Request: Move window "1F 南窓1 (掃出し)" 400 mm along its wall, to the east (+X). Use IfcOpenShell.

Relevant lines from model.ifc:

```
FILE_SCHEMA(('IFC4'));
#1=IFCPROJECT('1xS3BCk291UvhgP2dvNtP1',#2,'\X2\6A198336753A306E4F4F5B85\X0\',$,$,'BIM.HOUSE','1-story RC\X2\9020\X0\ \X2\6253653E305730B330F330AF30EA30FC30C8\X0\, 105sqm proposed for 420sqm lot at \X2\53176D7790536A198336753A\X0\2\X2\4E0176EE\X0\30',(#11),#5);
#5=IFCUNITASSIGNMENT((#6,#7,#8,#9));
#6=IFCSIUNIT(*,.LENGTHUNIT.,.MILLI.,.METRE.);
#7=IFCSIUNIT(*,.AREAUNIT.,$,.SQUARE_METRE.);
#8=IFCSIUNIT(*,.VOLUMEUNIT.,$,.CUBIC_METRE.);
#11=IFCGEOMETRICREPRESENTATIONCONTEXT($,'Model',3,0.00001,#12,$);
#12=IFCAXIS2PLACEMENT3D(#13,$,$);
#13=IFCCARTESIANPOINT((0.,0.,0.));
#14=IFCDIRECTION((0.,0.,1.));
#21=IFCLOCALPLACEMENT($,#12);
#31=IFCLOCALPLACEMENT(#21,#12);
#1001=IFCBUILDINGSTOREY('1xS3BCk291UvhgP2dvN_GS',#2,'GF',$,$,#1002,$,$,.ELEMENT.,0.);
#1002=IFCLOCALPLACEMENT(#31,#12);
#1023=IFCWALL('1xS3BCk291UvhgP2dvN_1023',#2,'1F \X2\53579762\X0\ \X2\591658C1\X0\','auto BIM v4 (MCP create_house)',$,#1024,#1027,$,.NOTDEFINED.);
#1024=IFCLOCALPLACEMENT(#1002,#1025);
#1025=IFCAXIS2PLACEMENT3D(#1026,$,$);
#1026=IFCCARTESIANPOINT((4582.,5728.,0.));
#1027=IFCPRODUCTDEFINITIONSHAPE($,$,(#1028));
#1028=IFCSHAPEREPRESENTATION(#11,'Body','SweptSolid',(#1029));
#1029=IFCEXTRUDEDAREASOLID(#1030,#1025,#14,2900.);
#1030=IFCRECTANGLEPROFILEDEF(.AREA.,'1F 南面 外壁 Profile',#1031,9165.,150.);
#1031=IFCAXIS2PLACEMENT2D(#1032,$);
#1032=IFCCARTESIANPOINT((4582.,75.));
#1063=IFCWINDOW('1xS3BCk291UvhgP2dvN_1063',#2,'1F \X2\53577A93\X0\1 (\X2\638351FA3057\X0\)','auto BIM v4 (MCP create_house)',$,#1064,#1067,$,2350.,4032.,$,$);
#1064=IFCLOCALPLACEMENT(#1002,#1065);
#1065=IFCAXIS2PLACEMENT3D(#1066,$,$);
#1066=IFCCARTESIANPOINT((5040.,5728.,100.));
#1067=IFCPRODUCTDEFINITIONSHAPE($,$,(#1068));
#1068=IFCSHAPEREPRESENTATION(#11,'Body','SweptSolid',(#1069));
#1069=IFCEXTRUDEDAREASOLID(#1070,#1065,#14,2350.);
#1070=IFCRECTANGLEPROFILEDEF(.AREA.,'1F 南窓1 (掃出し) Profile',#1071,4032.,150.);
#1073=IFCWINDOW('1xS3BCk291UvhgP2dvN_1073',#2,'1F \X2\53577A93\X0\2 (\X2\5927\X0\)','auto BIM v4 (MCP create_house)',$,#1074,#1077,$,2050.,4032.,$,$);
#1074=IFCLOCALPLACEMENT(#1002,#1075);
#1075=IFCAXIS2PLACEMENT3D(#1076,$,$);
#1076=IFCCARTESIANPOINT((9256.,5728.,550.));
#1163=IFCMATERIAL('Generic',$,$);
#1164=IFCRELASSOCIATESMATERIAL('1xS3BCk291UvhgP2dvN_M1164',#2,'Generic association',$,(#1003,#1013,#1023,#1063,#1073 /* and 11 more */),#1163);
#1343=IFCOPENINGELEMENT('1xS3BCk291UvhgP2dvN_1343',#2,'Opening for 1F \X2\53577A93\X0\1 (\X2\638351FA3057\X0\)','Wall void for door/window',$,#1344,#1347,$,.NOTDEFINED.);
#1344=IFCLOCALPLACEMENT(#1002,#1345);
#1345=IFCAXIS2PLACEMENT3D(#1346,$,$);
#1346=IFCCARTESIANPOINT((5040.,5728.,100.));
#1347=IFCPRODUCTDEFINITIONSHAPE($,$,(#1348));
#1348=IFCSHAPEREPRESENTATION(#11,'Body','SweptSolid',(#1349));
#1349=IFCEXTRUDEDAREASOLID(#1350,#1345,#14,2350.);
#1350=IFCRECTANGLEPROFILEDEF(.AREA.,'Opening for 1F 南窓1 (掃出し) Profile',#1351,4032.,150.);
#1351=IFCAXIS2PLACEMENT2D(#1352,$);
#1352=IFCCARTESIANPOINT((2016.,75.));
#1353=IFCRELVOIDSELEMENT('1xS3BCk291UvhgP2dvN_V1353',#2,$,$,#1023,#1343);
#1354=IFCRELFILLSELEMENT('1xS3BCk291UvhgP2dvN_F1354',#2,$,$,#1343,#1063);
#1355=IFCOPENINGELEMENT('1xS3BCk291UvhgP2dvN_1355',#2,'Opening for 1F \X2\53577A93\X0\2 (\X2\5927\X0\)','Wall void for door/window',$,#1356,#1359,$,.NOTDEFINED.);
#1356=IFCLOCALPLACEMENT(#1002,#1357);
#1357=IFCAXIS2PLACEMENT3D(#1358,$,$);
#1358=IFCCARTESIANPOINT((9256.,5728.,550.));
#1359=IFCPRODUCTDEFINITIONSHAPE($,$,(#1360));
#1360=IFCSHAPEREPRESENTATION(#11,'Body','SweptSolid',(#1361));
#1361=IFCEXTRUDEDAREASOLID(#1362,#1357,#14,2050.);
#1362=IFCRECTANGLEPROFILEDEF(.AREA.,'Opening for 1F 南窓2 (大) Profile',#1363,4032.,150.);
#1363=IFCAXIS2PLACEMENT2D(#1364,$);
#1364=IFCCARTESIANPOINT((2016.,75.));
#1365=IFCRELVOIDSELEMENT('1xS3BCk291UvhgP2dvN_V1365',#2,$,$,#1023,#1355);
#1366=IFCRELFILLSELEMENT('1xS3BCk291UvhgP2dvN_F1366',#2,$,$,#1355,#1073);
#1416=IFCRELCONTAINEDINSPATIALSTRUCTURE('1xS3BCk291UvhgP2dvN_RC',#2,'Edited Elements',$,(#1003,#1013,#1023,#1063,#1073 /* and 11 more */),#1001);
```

```python
import ifcopenshell
import ifcopenshell.api.geometry
import ifcopenshell.util.placement
import ifcopenshell.util.unit

model = ifcopenshell.open("model.ifc")
unit_scale = ifcopenshell.util.unit.calculate_unit_scale(model)

window = model.by_guid("1xS3BCk291UvhgP2dvN_1063")
opening = window.FillsVoids[0].RelatingOpeningElement
wall = opening.VoidsElements[0].RelatingBuildingElement

wall_matrix = ifcopenshell.util.placement.get_local_placement(wall.ObjectPlacement)
shift = wall_matrix[:3, 0] * 0.4 / unit_scale
before = ifcopenshell.util.placement.get_local_placement(window.ObjectPlacement)[:3, 3].copy()

# The window is not placed relative to its opening, so move both.
for product in (opening, window):
    matrix = ifcopenshell.util.placement.get_local_placement(product.ObjectPlacement)
    matrix[:3, 3] += shift
    ifcopenshell.api.geometry.edit_object_placement(model, product=product, matrix=matrix, is_si=False)

after = ifcopenshell.util.placement.get_local_placement(window.ObjectPlacement)[:3, 3]
print("window moved by", (after - before).round(3) + 0.0)

model.write("model_updated.ifc")
```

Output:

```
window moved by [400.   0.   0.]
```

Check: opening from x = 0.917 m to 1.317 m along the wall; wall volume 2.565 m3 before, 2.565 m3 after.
